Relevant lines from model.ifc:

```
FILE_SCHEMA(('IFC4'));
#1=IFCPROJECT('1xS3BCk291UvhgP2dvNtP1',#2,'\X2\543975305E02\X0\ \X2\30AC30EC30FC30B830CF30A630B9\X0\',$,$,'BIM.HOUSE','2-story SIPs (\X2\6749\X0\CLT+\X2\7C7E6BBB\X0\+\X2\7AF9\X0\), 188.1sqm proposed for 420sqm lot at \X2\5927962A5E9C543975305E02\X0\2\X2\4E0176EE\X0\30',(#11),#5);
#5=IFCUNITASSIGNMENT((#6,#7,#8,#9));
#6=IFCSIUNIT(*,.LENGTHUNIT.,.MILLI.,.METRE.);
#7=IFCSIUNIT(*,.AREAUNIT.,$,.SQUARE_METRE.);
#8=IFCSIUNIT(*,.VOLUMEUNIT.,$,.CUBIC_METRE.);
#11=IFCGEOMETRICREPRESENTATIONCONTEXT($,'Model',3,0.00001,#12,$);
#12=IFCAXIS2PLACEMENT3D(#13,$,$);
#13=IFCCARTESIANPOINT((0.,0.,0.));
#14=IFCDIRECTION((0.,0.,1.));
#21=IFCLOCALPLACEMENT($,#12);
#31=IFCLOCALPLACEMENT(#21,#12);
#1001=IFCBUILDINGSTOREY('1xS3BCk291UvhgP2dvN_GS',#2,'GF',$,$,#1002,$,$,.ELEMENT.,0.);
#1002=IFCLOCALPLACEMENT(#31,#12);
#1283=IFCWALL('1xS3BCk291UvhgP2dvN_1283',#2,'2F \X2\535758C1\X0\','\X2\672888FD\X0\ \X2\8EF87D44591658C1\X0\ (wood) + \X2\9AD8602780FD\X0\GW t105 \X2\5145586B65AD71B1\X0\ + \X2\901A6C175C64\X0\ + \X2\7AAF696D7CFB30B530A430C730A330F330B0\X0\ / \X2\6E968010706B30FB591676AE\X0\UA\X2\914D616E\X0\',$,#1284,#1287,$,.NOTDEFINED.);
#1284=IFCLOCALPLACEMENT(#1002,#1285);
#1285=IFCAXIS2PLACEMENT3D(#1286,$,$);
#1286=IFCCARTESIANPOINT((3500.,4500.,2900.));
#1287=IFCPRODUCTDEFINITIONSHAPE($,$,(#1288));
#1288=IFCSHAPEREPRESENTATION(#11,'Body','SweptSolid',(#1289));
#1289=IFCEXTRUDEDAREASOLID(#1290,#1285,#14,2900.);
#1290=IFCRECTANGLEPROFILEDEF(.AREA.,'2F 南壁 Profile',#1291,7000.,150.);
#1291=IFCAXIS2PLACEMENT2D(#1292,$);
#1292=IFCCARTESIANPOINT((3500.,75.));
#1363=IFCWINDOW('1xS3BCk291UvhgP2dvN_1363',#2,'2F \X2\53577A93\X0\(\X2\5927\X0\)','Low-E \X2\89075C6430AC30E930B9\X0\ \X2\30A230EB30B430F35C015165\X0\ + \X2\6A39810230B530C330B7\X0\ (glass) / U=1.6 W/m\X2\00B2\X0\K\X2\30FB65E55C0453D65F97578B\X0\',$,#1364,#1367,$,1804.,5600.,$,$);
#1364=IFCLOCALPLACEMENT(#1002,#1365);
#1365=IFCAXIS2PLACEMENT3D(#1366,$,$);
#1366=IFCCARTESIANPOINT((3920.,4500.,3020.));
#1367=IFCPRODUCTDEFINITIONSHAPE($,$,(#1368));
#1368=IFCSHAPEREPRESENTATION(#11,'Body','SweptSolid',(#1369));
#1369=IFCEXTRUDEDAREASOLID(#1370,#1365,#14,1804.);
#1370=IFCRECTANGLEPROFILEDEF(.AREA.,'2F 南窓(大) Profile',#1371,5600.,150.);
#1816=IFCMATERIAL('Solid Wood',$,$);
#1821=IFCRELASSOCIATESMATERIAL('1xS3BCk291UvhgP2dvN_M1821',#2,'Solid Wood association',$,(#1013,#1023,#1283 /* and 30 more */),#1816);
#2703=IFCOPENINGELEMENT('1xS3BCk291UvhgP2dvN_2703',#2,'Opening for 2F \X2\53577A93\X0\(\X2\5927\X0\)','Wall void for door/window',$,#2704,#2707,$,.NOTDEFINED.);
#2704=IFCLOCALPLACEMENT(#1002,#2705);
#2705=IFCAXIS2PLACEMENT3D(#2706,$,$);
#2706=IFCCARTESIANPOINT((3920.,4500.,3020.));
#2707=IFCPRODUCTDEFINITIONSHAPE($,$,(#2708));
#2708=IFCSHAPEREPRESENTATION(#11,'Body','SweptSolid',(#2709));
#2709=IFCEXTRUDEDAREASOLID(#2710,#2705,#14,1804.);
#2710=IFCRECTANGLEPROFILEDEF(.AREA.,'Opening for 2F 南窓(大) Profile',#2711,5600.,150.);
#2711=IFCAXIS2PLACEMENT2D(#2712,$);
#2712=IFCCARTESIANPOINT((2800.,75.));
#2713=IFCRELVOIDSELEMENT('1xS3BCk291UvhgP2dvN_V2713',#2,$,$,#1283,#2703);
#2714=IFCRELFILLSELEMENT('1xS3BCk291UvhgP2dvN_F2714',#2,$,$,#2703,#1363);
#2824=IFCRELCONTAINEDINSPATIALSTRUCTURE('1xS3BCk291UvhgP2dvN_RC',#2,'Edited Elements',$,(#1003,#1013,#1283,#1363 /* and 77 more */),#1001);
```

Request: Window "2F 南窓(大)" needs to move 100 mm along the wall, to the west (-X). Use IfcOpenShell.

```python
import ifcopenshell
import ifcopenshell.api.geometry
import ifcopenshell.util.placement

model = ifcopenshell.open("model.ifc")

window = model.by_guid("1xS3BCk291UvhgP2dvN_1363")
opening = window.FillsVoids[0].RelatingOpeningElement
wall = opening.VoidsElements[0].RelatingBuildingElement

wall_matrix = ifcopenshell.util.placement.get_local_placement(wall.ObjectPlacement)
shift = wall_matrix[:3, 0] * -100.0
before = ifcopenshell.util.placement.get_local_placement(window.ObjectPlacement)[:3, 3].copy()

# The window is not placed relative to its opening, so move both.
for product in (opening, window):
    matrix = ifcopenshell.util.placement.get_local_placement(product.ObjectPlacement)
    matrix[:3, 3] += shift
    ifcopenshell.api.geometry.edit_object_placement(model, product=product, matrix=matrix, is_si=False)

after = ifcopenshell.util.placement.get_local_placement(window.ObjectPlacement)[:3, 3]
print("window moved by", (after - before).round(3) + 0.0)

model.write("model-out.ifc")
```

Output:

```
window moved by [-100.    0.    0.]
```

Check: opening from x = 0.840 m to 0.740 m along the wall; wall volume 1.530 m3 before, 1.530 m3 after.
